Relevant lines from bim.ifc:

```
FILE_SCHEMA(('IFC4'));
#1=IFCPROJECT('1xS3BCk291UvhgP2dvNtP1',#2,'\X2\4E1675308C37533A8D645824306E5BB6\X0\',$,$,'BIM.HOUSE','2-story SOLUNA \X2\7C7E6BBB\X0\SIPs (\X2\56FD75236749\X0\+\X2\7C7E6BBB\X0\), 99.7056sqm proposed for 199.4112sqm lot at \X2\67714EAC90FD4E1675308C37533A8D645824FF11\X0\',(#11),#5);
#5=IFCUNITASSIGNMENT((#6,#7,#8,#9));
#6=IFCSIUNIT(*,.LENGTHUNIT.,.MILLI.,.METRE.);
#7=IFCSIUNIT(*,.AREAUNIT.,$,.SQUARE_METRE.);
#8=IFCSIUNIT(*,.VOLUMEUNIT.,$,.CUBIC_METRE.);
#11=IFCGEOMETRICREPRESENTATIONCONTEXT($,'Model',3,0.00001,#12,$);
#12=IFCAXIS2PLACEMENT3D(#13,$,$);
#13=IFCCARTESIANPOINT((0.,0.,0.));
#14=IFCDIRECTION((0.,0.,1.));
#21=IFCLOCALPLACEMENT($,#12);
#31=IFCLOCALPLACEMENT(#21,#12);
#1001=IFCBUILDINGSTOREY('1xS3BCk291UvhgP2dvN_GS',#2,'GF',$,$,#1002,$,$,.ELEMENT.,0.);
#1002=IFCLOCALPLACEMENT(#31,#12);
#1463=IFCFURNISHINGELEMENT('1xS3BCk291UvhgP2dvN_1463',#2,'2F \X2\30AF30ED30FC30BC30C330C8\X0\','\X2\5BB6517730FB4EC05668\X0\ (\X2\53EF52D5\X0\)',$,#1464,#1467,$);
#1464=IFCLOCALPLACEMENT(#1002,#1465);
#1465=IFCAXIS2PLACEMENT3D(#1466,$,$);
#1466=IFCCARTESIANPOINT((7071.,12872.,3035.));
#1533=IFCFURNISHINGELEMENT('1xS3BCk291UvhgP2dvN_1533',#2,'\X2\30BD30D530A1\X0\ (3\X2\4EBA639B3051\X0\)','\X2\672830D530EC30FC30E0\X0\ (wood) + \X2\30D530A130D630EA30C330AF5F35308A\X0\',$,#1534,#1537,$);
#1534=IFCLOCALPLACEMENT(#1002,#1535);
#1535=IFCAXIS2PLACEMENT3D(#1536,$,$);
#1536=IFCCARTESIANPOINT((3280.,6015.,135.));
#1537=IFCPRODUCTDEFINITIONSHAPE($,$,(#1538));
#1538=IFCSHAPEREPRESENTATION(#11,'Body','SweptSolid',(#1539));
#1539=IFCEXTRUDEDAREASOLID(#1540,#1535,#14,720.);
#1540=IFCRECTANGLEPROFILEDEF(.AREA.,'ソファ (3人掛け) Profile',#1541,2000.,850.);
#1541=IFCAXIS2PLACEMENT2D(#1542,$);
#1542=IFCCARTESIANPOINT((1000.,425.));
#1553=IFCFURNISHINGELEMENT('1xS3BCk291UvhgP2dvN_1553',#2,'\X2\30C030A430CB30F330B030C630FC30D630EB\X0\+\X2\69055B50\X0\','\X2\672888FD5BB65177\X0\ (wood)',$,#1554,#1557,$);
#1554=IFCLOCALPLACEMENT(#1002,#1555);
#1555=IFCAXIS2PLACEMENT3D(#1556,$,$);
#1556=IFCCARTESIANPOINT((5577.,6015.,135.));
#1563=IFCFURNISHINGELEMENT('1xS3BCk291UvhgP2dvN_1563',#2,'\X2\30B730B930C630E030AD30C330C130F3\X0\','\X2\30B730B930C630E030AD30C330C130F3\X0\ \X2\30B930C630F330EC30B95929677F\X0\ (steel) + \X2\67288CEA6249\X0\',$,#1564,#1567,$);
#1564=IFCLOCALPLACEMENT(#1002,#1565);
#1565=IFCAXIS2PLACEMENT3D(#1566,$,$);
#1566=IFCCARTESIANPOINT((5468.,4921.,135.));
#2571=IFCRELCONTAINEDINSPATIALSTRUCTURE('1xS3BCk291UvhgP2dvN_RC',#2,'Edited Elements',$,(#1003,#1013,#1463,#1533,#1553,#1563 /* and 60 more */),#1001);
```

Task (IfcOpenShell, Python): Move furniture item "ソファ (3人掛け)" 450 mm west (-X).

```python
import ifcopenshell
import ifcopenshell.api.geometry
import ifcopenshell.util.placement
import ifcopenshell.util.unit

model = ifcopenshell.open("bim.ifc")
unit_scale = ifcopenshell.util.unit.calculate_unit_scale(model)

item = model.by_guid("1xS3BCk291UvhgP2dvN_1533")
matrix = ifcopenshell.util.placement.get_local_placement(item.ObjectPlacement)
matrix[0, 3] -= 0.45 / unit_scale
ifcopenshell.api.geometry.edit_object_placement(model, product=item, matrix=matrix, is_si=False)

print(ifcopenshell.util.placement.get_local_placement(item.ObjectPlacement).round(3) + 0.0)

model.write("bim_edited.ifc")
```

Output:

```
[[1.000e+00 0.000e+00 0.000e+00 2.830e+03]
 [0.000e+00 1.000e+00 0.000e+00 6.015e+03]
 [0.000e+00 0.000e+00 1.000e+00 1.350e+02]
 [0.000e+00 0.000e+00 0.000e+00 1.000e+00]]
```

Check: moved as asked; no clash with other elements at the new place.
